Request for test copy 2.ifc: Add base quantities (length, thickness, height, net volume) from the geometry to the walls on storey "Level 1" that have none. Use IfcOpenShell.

First a look at what the model holds.

```python
import ifcopenshell
import ifcopenshell.util.element
import ifcopenshell.util.unit

model = ifcopenshell.open("test copy 2.ifc")
print(model.schema)
for unit_type in ("LENGTHUNIT", "AREAUNIT", "VOLUMEUNIT"):
    print(unit_type, ifcopenshell.util.unit.calculate_unit_scale(model, unit_type))
storey = next(s for s in model.by_type("IfcBuildingStorey") if s.Name == "Level 1")
walls = [e for e in ifcopenshell.util.element.get_decomposition(storey) if e.is_a("IfcWall")]
for e in sorted(walls, key=lambda e: e.id()):
    print(e.id(), e.is_a(), e.Name, list(ifcopenshell.util.element.get_psets(e, qtos_only=True)), sep=" | ")
```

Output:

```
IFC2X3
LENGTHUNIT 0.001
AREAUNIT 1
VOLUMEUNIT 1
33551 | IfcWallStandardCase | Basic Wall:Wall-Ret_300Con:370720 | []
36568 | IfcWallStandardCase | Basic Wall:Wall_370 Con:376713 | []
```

```python
import ifcopenshell
import ifcopenshell.api.pset
import ifcopenshell.geom
import ifcopenshell.util.element
import ifcopenshell.util.shape
import ifcopenshell.util.unit

model = ifcopenshell.open("test copy 2.ifc")
unit_scale = ifcopenshell.util.unit.calculate_unit_scale(model)
volume_scale = ifcopenshell.util.unit.calculate_unit_scale(model, "VOLUMEUNIT")
settings = ifcopenshell.geom.settings()

storey = next(s for s in model.by_type("IfcBuildingStorey") if s.Name == "Level 1")
walls = [e for e in ifcopenshell.util.element.get_decomposition(storey) if e.is_a("IfcWall")]

for e in sorted(walls, key=lambda e: e.id()):
    if ifcopenshell.util.element.get_psets(e, qtos_only=True, should_inherit=False):
        continue
    # Geometry comes back in metres, in the element's own axes.
    shape = ifcopenshell.geom.create_shape(settings, e)
    values = {
        "Length": ifcopenshell.util.shape.get_x(shape.geometry) / unit_scale,
        "Width": ifcopenshell.util.shape.get_y(shape.geometry) / unit_scale,
        "Height": ifcopenshell.util.shape.get_z(shape.geometry) / unit_scale,
        "NetVolume": ifcopenshell.util.shape.get_volume(shape.geometry) / volume_scale,
    }
    qto = ifcopenshell.api.pset.add_qto(model, product=e, name="BaseQuantities")
    ifcopenshell.api.pset.edit_qto(model, qto=qto, properties=values)
    print(e.id(), {k: round(v, 3) for k, v in values.items()})

model.write("test copy 2_v2.ifc")
```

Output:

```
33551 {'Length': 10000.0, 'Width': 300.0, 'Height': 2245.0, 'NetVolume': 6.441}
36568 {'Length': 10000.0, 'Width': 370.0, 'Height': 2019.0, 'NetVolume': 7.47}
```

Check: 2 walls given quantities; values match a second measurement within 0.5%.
